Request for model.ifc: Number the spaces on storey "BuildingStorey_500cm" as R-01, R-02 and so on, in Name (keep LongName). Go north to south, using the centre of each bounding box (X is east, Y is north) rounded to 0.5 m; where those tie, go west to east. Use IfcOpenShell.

First a look at what the model holds.

```python
import ifcopenshell
import ifcopenshell.util.element
import ifcopenshell.util.placement

model = ifcopenshell.open("model.ifc")
print(model.schema)
storey = next(s for s in model.by_type("IfcBuildingStorey") if s.Name == "BuildingStorey_500cm")
spaces = [e for e in ifcopenshell.util.element.get_decomposition(storey) if e.is_a("IfcSpace")]
for e in sorted(spaces, key=lambda e: e.id()):
    origin = ifcopenshell.util.placement.get_local_placement(e.ObjectPlacement)[:3, 3]
    print(e.id(), e.Name, e.LongName, origin.round(2) + 0.0, sep=" | ")
```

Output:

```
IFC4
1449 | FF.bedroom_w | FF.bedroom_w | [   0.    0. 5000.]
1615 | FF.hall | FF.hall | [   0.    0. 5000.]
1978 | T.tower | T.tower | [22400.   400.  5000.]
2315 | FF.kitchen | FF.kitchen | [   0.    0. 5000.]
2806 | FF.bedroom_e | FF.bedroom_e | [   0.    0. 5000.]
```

```python
import ifcopenshell
import ifcopenshell.geom
import ifcopenshell.util.element
import ifcopenshell.util.shape

model = ifcopenshell.open("model.ifc")
settings = ifcopenshell.geom.settings()
settings.set("use-world-coords", True)


def centre(element):
    shape = ifcopenshell.geom.create_shape(settings, element)
    return ifcopenshell.util.shape.get_bbox_centroid(shape.geometry)


storey = next(s for s in model.by_type("IfcBuildingStorey") if s.Name == "BuildingStorey_500cm")
spaces = [e for e in ifcopenshell.util.element.get_decomposition(storey) if e.is_a("IfcSpace")]

# Insertion points can sit at a corner or the storey origin, so sort by the geometry (in metres).
centres = {e: centre(e) for e in spaces}
spaces.sort(key=lambda e: (-round(centres[e][1] / 0.5), centres[e][0]))

for i, e in enumerate(spaces, start=1):
    number = f"R-{i:02d}"
    e.Name = number
    print(e.id(), number)

model.write("model_v2.ifc")
```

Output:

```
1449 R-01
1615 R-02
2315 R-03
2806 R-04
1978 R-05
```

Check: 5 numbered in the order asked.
